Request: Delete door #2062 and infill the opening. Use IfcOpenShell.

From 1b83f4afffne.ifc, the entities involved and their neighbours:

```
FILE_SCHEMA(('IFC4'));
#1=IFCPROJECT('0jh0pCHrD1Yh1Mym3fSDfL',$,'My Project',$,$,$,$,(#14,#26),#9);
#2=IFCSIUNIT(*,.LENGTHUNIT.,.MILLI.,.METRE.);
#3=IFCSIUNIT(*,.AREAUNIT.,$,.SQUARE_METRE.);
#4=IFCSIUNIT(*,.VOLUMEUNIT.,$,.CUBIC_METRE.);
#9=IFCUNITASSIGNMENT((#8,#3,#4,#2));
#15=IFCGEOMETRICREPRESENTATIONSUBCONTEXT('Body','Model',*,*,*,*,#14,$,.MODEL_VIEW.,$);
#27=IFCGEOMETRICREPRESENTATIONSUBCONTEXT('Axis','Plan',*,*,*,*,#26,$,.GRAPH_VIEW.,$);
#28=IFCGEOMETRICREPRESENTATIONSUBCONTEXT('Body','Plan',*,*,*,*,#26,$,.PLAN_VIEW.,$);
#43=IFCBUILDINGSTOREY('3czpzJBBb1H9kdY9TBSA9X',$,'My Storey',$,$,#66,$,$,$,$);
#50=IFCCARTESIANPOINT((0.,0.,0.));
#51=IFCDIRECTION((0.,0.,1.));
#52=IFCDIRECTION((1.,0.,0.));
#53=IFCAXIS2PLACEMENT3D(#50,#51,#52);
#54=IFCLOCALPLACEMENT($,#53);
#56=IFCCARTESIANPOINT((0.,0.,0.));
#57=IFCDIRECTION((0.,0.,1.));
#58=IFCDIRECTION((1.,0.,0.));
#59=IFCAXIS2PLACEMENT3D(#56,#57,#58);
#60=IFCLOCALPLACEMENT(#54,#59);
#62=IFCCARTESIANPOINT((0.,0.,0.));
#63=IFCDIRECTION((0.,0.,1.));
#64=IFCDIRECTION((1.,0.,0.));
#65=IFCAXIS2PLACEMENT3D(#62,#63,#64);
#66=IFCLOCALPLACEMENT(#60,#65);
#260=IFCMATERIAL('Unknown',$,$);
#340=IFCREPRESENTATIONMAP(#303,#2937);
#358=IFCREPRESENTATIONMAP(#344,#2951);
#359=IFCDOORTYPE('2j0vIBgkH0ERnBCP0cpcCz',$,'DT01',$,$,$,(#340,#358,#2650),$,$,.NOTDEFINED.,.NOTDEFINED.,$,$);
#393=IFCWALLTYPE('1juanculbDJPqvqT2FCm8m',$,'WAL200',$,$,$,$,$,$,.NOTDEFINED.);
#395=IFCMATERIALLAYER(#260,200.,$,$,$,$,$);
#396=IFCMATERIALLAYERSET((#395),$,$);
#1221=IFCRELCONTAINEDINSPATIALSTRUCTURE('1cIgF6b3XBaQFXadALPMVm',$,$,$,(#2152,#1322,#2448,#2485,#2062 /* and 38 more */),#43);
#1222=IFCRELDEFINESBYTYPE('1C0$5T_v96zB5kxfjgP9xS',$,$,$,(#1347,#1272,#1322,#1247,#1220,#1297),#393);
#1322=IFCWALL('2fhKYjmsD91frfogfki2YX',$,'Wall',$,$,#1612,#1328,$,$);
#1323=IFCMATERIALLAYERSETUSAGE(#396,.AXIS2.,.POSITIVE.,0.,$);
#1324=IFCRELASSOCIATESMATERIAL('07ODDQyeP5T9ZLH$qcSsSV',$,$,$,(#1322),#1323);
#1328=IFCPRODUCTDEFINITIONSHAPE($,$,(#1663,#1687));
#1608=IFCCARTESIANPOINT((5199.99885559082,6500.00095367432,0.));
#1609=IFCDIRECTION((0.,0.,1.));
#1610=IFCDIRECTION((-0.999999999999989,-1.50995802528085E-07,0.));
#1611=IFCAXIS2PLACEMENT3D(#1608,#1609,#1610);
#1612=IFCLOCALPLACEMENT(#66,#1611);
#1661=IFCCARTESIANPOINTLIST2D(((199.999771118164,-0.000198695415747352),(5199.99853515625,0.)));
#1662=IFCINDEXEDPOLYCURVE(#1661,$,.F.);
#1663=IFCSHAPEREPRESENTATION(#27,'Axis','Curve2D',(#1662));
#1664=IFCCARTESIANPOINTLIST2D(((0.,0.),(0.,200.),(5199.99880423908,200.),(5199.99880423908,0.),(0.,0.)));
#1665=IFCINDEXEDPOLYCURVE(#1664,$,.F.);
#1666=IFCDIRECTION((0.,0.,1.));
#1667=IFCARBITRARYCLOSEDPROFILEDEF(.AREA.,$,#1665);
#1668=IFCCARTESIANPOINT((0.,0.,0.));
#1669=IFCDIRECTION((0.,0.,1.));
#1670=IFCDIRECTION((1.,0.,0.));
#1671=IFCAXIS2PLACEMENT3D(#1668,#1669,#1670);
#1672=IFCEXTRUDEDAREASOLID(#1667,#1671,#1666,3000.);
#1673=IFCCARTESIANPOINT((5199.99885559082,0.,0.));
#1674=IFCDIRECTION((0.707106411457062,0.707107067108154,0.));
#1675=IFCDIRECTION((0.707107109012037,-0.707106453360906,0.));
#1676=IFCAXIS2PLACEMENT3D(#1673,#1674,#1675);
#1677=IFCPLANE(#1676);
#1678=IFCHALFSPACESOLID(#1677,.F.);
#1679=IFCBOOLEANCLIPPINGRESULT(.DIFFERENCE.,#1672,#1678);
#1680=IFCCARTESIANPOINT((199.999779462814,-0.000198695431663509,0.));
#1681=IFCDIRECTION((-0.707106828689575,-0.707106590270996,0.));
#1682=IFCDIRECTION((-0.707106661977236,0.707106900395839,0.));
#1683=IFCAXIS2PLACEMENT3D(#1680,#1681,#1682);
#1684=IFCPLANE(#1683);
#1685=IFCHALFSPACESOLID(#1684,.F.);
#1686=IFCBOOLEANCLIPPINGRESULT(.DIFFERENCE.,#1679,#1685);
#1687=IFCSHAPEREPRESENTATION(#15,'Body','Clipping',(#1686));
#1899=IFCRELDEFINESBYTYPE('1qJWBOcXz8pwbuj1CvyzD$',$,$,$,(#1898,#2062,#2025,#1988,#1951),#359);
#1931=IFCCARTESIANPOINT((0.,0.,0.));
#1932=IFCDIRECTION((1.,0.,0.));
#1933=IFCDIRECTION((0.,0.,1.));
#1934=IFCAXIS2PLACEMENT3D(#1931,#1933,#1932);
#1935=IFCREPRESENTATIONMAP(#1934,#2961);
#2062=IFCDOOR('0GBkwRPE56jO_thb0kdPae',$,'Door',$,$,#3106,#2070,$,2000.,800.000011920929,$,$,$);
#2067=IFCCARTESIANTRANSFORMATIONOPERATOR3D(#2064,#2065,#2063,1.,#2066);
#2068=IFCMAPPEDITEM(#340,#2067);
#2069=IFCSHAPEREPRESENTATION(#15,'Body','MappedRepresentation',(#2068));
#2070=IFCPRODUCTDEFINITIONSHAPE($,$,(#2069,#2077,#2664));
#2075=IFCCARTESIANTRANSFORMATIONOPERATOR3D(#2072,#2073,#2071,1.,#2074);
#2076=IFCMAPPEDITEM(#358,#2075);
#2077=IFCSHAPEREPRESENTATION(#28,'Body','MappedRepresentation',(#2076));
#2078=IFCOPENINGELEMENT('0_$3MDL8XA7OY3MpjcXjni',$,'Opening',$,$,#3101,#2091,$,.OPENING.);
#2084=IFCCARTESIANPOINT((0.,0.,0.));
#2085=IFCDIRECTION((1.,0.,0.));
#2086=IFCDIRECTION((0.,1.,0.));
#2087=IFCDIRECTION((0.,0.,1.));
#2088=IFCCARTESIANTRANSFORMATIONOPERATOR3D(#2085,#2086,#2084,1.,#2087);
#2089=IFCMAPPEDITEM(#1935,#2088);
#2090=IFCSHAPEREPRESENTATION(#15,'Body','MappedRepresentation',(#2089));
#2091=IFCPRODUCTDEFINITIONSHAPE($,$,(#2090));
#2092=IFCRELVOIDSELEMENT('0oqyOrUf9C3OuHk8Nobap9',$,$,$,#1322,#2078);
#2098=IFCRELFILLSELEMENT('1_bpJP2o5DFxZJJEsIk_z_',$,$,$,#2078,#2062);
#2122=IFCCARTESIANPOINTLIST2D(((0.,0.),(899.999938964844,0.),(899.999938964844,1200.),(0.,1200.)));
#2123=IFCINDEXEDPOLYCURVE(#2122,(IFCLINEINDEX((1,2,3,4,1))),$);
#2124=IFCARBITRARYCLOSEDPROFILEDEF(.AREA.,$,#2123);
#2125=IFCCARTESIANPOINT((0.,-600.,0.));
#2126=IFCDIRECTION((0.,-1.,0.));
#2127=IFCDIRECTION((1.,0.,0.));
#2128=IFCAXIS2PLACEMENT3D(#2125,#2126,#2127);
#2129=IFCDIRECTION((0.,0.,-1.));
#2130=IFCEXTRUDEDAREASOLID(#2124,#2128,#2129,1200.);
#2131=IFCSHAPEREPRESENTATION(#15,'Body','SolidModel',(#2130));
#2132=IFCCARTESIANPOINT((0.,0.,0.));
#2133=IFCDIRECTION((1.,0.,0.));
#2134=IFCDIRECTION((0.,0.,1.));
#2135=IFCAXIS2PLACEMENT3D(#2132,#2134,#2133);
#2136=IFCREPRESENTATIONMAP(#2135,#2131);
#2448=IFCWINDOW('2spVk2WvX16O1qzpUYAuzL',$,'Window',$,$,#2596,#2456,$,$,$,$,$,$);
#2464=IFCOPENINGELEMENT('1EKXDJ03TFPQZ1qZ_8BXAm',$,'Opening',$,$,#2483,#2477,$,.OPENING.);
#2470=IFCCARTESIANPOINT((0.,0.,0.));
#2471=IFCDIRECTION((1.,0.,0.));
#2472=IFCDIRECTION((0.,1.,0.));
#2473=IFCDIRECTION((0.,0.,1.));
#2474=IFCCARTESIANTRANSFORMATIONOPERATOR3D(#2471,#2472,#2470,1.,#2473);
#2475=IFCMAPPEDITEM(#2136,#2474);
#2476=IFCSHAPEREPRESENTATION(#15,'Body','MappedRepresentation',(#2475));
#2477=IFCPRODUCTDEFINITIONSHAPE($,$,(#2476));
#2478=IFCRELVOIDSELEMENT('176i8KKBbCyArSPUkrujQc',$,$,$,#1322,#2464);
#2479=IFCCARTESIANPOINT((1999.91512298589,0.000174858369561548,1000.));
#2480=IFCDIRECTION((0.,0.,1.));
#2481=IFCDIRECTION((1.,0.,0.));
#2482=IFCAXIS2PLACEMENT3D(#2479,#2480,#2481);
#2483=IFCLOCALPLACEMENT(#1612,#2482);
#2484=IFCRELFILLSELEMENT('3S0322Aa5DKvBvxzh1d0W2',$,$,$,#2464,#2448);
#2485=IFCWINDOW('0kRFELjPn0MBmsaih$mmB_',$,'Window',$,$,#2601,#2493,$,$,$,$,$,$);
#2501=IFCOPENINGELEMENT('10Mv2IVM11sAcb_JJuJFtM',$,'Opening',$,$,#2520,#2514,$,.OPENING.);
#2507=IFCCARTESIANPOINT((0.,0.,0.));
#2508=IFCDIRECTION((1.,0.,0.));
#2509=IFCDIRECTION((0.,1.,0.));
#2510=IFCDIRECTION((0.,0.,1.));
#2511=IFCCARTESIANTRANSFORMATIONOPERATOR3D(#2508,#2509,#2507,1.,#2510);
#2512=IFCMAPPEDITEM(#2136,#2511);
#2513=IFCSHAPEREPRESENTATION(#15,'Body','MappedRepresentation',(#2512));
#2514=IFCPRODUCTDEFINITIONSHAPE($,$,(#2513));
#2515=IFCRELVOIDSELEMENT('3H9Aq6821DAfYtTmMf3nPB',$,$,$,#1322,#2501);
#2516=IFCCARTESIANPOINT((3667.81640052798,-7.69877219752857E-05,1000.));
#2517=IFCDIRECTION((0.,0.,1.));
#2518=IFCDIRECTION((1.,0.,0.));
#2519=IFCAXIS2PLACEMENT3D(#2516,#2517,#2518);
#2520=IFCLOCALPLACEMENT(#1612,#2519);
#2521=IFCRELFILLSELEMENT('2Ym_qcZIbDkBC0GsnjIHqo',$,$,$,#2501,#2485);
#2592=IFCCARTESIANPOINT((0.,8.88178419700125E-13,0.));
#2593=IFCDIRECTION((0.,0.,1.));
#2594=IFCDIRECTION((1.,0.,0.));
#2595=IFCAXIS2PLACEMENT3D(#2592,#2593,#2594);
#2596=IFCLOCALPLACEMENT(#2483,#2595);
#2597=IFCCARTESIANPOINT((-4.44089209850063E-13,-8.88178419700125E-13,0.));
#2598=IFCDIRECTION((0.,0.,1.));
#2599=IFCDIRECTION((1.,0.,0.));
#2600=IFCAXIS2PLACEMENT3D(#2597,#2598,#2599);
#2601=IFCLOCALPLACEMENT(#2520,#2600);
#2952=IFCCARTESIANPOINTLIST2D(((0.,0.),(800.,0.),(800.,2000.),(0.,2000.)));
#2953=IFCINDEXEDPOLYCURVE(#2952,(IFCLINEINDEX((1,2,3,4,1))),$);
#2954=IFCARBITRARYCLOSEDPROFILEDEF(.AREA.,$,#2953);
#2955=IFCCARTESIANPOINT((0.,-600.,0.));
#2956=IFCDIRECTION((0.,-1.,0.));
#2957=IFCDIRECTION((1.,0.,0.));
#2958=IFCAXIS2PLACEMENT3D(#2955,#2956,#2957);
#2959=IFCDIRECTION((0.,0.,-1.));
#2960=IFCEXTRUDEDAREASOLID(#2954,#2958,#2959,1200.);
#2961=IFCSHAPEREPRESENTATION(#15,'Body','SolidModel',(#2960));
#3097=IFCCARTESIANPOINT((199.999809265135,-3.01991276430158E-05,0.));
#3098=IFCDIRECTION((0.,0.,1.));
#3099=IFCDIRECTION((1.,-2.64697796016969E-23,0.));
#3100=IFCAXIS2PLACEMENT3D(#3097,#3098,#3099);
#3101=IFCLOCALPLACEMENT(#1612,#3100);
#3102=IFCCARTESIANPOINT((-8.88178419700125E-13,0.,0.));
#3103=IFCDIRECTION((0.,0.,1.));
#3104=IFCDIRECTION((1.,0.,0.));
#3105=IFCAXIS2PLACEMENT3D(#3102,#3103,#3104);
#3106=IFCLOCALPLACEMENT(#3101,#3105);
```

```python
import ifcopenshell
import ifcopenshell.api.feature
import ifcopenshell.api.root
import ifcopenshell.geom
import ifcopenshell.util.shape

model = ifcopenshell.open("1b83f4afffne.ifc")
settings = ifcopenshell.geom.settings()


def volume(element):
    """Net volume in cubic metres, openings subtracted."""
    shape = ifcopenshell.geom.create_shape(settings, element)
    return ifcopenshell.util.shape.get_volume(shape.geometry)


door = model.by_id(2062)
opening = door.FillsVoids[0].RelatingOpeningElement
wall = opening.VoidsElements[0].RelatingBuildingElement
before = volume(wall)

ifcopenshell.api.root.remove_product(model, product=door)
ifcopenshell.api.feature.remove_feature(model, feature=opening)

after = volume(wall)

print(f"wall volume {before:.3f} -> {after:.3f} m3")

model.write("1b83f4afffne_updated.ifc")
```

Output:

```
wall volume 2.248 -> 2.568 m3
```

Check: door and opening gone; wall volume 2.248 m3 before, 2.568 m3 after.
